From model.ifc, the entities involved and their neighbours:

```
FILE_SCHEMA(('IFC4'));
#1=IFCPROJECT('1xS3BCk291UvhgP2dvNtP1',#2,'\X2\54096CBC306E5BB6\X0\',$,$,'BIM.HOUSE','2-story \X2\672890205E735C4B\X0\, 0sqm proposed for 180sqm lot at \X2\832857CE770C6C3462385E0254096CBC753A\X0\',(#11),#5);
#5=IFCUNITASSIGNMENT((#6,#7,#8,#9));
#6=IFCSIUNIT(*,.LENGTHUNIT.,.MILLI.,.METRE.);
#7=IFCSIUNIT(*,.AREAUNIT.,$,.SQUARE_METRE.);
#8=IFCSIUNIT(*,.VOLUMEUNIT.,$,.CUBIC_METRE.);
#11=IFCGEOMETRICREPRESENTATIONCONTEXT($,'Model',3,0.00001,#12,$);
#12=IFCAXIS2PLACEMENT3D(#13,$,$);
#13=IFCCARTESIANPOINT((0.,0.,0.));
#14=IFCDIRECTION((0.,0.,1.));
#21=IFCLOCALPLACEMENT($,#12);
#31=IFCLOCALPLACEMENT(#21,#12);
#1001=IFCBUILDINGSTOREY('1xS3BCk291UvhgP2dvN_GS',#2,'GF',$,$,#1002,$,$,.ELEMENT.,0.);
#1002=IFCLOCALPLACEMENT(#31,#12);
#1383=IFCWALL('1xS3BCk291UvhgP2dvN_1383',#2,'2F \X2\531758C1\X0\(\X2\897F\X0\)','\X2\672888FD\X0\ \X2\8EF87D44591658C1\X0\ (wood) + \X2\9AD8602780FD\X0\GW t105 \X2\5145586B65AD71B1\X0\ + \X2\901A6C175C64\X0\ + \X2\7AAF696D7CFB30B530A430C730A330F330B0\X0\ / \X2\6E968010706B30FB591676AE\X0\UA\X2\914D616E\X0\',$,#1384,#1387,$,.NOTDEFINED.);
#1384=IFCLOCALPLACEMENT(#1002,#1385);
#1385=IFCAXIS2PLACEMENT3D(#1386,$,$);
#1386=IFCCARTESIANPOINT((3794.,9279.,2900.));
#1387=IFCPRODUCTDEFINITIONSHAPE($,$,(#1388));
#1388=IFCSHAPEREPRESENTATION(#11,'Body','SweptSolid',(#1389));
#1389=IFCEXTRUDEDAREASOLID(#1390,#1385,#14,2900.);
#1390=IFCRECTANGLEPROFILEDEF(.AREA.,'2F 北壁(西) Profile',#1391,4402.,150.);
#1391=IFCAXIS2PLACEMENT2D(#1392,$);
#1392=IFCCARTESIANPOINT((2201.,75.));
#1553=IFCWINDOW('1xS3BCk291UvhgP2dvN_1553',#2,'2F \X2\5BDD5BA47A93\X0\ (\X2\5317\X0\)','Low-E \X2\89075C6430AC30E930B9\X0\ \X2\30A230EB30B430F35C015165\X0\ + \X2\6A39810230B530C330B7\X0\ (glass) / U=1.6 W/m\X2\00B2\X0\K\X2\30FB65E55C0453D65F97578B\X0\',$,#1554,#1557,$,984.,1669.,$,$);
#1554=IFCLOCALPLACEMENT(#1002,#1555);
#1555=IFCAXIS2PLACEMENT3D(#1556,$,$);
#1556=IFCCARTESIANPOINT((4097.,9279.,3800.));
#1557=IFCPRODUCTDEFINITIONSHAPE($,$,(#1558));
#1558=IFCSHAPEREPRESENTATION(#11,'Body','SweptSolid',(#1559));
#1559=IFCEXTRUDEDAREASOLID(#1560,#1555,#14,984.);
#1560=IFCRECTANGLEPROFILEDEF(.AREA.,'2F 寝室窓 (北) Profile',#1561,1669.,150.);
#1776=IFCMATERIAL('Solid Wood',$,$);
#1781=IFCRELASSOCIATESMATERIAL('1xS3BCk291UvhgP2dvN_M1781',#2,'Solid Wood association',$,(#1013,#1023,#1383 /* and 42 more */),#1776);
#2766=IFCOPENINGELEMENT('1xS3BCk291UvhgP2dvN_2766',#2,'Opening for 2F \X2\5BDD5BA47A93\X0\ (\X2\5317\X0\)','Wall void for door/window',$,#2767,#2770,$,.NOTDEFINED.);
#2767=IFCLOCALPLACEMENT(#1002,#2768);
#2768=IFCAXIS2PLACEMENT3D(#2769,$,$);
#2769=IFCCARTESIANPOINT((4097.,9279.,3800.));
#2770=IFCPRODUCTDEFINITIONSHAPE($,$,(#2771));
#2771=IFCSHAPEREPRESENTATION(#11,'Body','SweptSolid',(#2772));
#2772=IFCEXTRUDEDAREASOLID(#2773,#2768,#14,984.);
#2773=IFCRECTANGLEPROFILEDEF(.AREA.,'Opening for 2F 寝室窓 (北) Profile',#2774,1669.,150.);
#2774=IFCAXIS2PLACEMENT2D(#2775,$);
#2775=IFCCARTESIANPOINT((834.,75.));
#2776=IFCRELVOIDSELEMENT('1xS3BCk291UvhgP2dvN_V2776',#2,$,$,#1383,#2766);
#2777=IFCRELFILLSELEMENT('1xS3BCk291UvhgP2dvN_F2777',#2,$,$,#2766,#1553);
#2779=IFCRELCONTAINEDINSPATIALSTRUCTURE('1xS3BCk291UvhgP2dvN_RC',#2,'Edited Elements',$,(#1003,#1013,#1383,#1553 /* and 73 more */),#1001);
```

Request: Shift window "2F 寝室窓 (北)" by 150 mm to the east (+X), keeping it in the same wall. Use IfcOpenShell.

```python
import ifcopenshell
import ifcopenshell.api.geometry
import ifcopenshell.util.placement

model = ifcopenshell.open("model.ifc")

window = model.by_id(1553)
opening = window.FillsVoids[0].RelatingOpeningElement
wall = opening.VoidsElements[0].RelatingBuildingElement

wall_matrix = ifcopenshell.util.placement.get_local_placement(wall.ObjectPlacement)
shift = wall_matrix[:3, 0] * 150.0
before = ifcopenshell.util.placement.get_local_placement(window.ObjectPlacement)[:3, 3].copy()

# The window is not placed relative to its opening, so move both.
for product in (opening, window):
    matrix = ifcopenshell.util.placement.get_local_placement(product.ObjectPlacement)
    matrix[:3, 3] += shift
    ifcopenshell.api.geometry.edit_object_placement(model, product=product, matrix=matrix, is_si=False)

after = ifcopenshell.util.placement.get_local_placement(window.ObjectPlacement)[:3, 3]
print("window moved by", (after - before).round(3) + 0.0)

model.write("model_edited.ifc")
```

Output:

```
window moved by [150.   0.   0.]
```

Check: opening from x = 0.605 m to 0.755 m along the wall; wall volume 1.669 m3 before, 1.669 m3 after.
